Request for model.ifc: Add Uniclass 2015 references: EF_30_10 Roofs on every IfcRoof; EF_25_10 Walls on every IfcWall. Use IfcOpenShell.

First a look at what the model holds.

```python
import ifcopenshell

model = ifcopenshell.open("model.ifc")
print(model.schema)
print("classifications:", [c.Name for c in model.by_type("IfcClassification")])
for ifc_class in ("IfcDoor", "IfcRoof", "IfcStair", "IfcWall", "IfcWindow"):
    print(ifc_class, len(model.by_type(ifc_class)))
```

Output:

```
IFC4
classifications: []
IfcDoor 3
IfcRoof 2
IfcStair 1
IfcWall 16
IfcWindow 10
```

```python
import ifcopenshell
import ifcopenshell.api.classification

model = ifcopenshell.open("model.ifc")

system = ifcopenshell.api.classification.add_classification(model, classification="Uniclass 2015")

codes = {
    "IfcRoof": ("EF_30_10", "Roofs"),
    "IfcWall": ("EF_25_10", "Walls"),
}
for ifc_class, (code, name) in codes.items():
    products = model.by_type(ifc_class)
    ifcopenshell.api.classification.add_reference(
        model, products=products, classification=system, identification=code, name=name
    )
    print(code, len(products))

model.write("model-out.ifc")
```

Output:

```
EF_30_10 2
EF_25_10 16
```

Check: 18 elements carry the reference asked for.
